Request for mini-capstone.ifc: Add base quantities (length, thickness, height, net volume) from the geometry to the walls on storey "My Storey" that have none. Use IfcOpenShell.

First a look at what the model holds.

```python
import ifcopenshell
import ifcopenshell.util.element
import ifcopenshell.util.unit

model = ifcopenshell.open("mini-capstone.ifc")
print(model.schema)
for unit_type in ("LENGTHUNIT", "AREAUNIT", "VOLUMEUNIT"):
    print(unit_type, ifcopenshell.util.unit.calculate_unit_scale(model, unit_type))
storey = next(s for s in model.by_type("IfcBuildingStorey") if s.Name == "My Storey")
walls = [e for e in ifcopenshell.util.element.get_decomposition(storey) if e.is_a("IfcWall")]
for e in sorted(walls, key=lambda e: e.id()):
    print(e.id(), e.is_a(), e.Name, list(ifcopenshell.util.element.get_psets(e, qtos_only=True)), sep=" | ")
```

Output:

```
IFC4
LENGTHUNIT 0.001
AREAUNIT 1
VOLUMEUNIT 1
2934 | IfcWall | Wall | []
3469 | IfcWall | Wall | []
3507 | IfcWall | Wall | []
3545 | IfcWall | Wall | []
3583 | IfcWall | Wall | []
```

```python
import ifcopenshell
import ifcopenshell.api.pset
import ifcopenshell.geom
import ifcopenshell.util.element
import ifcopenshell.util.shape
import ifcopenshell.util.unit

model = ifcopenshell.open("mini-capstone.ifc")
unit_scale = ifcopenshell.util.unit.calculate_unit_scale(model)
volume_scale = ifcopenshell.util.unit.calculate_unit_scale(model, "VOLUMEUNIT")
settings = ifcopenshell.geom.settings()

storey = next(s for s in model.by_type("IfcBuildingStorey") if s.Name == "My Storey")
walls = [e for e in ifcopenshell.util.element.get_decomposition(storey) if e.is_a("IfcWall")]

for e in sorted(walls, key=lambda e: e.id()):
    if ifcopenshell.util.element.get_psets(e, qtos_only=True, should_inherit=False):
        continue
    # Geometry comes back in metres, in the element's own axes.
    shape = ifcopenshell.geom.create_shape(settings, e)
    values = {
        "Length": ifcopenshell.util.shape.get_x(shape.geometry) / unit_scale,
        "Width": ifcopenshell.util.shape.get_y(shape.geometry) / unit_scale,
        "Height": ifcopenshell.util.shape.get_z(shape.geometry) / unit_scale,
        "NetVolume": ifcopenshell.util.shape.get_volume(shape.geometry) / volume_scale,
    }
    qto = ifcopenshell.api.pset.add_qto(model, product=e, name="Qto_WallBaseQuantities")
    ifcopenshell.api.pset.edit_qto(model, qto=qto, properties=values)
    print(e.id(), {k: round(v, 3) for k, v in values.items()})

model.write("mini-capstone_updated.ifc")
```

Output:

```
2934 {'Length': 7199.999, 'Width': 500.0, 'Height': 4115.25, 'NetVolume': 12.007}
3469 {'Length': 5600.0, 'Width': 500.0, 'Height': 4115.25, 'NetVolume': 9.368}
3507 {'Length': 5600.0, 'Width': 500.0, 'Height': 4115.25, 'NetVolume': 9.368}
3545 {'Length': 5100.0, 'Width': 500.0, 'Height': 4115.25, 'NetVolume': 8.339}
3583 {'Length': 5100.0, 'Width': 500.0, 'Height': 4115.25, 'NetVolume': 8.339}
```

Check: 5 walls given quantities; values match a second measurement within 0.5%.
